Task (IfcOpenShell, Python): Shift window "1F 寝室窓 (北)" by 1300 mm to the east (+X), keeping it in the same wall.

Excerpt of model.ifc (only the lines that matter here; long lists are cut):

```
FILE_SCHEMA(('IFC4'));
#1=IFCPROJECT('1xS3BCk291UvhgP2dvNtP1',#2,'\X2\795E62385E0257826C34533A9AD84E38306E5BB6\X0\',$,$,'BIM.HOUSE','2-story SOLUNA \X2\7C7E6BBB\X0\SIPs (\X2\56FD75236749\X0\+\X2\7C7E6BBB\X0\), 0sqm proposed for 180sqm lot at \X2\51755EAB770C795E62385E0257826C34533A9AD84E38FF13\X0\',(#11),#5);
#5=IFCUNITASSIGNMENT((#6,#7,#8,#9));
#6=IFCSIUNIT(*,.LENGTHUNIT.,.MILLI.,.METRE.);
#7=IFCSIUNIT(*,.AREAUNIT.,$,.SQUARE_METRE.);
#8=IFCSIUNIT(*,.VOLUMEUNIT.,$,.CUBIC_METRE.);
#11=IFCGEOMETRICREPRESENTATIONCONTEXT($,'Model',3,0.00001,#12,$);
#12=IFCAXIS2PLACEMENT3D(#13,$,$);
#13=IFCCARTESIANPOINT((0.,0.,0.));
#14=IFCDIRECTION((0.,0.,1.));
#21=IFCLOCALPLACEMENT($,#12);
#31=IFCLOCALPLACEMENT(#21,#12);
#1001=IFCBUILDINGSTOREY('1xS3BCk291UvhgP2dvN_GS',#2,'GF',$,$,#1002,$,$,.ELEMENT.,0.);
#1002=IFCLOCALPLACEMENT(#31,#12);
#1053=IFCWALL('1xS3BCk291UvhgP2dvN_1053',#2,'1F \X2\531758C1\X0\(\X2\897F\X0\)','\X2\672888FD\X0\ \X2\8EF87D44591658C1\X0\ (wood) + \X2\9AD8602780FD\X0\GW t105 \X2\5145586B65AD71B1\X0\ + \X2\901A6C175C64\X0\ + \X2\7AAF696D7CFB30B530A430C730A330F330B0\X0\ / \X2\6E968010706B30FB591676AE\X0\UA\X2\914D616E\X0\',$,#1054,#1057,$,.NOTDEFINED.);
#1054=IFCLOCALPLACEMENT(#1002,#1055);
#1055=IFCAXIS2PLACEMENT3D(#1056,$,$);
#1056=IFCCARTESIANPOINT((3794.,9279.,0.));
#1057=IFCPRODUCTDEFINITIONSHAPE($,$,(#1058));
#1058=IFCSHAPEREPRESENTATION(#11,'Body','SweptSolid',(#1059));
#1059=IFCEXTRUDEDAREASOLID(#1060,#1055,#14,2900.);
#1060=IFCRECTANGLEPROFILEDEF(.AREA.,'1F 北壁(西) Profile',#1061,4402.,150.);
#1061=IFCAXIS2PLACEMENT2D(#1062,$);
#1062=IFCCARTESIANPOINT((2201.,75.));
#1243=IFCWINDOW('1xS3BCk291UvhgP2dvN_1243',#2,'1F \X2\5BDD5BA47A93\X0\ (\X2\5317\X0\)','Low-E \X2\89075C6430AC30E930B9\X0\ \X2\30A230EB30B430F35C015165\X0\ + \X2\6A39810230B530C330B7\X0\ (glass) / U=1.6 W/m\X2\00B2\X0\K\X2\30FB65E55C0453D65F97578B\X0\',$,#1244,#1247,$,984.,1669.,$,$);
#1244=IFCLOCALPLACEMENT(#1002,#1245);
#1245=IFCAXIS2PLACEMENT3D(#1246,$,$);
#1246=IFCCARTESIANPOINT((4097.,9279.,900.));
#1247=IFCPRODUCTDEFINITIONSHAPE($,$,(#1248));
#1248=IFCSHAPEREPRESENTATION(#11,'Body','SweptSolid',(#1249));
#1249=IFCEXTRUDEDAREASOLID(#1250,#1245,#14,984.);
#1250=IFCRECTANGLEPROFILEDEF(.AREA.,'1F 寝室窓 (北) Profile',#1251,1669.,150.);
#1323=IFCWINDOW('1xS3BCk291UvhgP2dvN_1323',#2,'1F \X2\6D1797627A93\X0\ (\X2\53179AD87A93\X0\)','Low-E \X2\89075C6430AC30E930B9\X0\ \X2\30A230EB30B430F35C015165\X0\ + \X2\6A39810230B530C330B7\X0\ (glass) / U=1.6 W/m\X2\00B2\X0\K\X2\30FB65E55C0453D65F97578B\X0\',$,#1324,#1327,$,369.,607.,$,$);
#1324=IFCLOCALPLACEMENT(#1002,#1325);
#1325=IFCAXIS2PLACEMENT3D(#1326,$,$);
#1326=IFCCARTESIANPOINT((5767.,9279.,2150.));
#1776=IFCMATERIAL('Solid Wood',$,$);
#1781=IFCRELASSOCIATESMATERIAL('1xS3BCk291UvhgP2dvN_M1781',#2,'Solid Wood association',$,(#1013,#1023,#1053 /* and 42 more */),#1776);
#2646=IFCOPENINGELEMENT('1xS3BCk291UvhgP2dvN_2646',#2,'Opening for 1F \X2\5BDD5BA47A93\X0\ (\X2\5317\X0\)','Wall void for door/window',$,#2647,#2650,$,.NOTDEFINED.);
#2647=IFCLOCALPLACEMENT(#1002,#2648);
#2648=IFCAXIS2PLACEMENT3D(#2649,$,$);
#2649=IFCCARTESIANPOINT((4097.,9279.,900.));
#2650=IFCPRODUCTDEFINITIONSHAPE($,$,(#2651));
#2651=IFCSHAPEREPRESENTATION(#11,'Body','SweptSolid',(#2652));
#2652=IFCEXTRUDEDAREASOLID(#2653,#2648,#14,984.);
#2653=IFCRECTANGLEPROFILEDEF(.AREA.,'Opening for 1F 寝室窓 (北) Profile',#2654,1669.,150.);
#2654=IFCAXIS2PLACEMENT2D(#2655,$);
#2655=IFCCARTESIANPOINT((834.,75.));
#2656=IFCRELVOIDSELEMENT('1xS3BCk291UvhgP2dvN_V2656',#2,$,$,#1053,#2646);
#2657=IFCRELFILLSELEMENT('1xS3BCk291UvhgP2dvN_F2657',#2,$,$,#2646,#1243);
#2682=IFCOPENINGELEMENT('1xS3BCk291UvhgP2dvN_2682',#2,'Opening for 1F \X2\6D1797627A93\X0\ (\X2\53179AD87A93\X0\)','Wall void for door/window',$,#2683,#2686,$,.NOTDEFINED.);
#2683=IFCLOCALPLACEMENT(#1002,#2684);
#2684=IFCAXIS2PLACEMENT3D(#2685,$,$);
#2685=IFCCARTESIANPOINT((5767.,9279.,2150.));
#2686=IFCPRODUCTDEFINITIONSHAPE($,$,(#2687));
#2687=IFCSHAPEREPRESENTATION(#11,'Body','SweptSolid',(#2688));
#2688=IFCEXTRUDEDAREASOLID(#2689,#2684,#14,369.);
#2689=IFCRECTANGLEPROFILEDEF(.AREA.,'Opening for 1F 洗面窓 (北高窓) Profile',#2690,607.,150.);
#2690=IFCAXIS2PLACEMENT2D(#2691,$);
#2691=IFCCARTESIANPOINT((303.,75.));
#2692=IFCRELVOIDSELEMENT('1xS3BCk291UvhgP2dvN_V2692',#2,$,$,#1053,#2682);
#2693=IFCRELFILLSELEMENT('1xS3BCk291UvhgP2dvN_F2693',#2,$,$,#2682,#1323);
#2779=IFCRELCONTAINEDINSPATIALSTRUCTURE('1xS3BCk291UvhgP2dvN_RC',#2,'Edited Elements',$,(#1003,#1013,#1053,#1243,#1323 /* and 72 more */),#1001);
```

```python
import ifcopenshell
import ifcopenshell.api.geometry
import ifcopenshell.util.placement

model = ifcopenshell.open("model.ifc")

window = model.by_id(1243)
opening = window.FillsVoids[0].RelatingOpeningElement
wall = opening.VoidsElements[0].RelatingBuildingElement

wall_matrix = ifcopenshell.util.placement.get_local_placement(wall.ObjectPlacement)
shift = wall_matrix[:3, 0] * 1300.0
before = ifcopenshell.util.placement.get_local_placement(window.ObjectPlacement)[:3, 3].copy()

# The window is not placed relative to its opening, so move both.
for product in (opening, window):
    matrix = ifcopenshell.util.placement.get_local_placement(product.ObjectPlacement)
    matrix[:3, 3] += shift
    ifcopenshell.api.geometry.edit_object_placement(model, product=product, matrix=matrix, is_si=False)

after = ifcopenshell.util.placement.get_local_placement(window.ObjectPlacement)[:3, 3]
print("window moved by", (after - before).round(3) + 0.0)

model.write("model-out.ifc")
```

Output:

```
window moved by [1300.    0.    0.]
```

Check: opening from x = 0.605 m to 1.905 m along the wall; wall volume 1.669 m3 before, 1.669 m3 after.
